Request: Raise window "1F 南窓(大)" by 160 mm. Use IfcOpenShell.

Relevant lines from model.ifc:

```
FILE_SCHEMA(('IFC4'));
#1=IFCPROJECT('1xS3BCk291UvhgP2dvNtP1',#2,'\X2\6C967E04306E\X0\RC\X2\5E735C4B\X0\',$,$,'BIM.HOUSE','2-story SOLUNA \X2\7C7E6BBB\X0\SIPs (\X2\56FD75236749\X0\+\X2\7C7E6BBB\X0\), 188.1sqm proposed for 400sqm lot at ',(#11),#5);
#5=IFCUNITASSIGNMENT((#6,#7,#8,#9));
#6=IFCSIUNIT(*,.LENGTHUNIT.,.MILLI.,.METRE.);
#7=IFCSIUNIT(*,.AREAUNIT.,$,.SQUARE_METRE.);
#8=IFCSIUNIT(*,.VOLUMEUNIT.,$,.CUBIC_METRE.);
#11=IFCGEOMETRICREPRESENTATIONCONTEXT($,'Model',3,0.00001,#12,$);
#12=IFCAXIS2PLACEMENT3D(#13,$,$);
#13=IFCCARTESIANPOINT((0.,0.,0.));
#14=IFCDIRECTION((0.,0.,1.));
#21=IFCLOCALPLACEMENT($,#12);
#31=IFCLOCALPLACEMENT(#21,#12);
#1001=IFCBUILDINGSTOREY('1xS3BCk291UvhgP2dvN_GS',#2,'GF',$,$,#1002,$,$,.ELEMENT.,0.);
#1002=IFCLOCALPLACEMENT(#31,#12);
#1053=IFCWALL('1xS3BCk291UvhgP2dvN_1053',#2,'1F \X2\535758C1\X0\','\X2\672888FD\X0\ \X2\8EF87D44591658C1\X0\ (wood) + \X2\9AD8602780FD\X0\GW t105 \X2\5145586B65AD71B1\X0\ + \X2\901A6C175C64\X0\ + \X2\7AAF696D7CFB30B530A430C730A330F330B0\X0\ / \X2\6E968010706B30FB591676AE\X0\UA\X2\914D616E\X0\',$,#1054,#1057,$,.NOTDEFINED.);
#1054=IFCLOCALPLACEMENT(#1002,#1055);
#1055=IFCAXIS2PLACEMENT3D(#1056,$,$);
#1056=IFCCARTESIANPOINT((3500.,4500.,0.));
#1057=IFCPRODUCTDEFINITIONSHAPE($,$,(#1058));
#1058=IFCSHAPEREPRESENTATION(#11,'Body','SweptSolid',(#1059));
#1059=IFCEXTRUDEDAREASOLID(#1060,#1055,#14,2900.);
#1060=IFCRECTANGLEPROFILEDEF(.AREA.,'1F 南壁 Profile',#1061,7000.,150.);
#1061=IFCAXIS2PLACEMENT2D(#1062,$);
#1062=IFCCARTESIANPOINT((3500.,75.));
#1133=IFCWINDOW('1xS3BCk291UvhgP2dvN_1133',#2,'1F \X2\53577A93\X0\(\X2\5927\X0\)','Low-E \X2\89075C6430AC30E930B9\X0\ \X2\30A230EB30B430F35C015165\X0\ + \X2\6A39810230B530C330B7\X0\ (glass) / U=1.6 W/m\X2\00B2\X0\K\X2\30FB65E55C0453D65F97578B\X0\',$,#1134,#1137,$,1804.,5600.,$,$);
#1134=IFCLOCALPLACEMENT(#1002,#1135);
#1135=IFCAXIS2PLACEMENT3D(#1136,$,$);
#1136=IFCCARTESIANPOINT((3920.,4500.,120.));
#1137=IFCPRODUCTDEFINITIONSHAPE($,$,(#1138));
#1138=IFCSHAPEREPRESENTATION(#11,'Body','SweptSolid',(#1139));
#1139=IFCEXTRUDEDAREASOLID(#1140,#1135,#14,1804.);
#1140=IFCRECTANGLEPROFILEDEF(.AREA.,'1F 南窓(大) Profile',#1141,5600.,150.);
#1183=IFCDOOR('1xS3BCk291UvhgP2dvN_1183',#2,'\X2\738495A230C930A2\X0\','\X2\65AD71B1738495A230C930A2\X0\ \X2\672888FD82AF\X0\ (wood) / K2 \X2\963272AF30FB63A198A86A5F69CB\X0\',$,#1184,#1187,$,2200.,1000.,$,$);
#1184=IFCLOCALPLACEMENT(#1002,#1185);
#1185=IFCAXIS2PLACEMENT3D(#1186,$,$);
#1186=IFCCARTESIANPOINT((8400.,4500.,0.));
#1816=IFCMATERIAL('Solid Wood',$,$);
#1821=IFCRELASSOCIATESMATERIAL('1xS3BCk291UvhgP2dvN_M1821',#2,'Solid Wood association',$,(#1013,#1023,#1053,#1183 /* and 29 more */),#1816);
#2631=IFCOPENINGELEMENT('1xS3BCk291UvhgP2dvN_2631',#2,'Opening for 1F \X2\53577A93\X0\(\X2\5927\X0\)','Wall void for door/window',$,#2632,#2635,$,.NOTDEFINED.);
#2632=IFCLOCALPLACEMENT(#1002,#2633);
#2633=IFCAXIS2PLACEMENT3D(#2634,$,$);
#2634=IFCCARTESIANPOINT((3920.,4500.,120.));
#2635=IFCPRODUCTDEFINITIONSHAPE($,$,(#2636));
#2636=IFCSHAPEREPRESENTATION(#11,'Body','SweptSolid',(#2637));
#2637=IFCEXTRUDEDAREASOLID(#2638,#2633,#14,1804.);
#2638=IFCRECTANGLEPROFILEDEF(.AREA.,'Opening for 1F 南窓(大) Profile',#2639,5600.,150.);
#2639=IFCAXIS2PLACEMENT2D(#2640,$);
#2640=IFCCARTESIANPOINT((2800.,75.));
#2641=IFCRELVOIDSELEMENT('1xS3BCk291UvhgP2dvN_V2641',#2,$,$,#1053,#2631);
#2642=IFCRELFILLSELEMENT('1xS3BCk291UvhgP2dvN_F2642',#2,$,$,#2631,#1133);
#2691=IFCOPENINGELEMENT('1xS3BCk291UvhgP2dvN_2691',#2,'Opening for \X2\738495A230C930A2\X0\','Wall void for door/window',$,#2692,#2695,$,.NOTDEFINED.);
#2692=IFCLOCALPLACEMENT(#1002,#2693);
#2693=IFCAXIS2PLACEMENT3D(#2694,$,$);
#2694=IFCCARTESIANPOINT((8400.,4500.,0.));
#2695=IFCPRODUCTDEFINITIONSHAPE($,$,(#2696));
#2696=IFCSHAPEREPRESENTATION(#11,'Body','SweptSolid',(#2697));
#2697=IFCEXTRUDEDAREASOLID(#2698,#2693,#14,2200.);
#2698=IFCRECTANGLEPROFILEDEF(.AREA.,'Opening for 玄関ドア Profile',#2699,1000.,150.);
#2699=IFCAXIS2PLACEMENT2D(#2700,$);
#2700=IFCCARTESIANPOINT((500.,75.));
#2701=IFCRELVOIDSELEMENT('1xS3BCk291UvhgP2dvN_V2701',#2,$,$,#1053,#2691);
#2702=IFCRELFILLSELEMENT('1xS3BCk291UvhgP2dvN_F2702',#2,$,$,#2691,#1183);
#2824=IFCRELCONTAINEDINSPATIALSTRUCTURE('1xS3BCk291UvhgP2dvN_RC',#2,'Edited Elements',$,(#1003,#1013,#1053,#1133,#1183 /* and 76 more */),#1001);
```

```python
import numpy as np
import ifcopenshell
import ifcopenshell.api.geometry
import ifcopenshell.util.placement
import ifcopenshell.util.unit

model = ifcopenshell.open("model.ifc")
unit_scale = ifcopenshell.util.unit.calculate_unit_scale(model)

window = model.by_guid("1xS3BCk291UvhgP2dvN_1133")
opening = window.FillsVoids[0].RelatingOpeningElement
dz = 0.16 / unit_scale

shift = np.array([0.0, 0.0, dz])
# The window is not placed relative to its opening, so move both.
for product in (opening, window):
    matrix = ifcopenshell.util.placement.get_local_placement(product.ObjectPlacement)
    matrix[:3, 3] += shift
    ifcopenshell.api.geometry.edit_object_placement(model, product=product, matrix=matrix, is_si=False)

print(f"moved by {dz * unit_scale:+.3f} m")

model.write("model_rev.ifc")
```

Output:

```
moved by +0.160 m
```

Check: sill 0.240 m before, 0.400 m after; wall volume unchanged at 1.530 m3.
